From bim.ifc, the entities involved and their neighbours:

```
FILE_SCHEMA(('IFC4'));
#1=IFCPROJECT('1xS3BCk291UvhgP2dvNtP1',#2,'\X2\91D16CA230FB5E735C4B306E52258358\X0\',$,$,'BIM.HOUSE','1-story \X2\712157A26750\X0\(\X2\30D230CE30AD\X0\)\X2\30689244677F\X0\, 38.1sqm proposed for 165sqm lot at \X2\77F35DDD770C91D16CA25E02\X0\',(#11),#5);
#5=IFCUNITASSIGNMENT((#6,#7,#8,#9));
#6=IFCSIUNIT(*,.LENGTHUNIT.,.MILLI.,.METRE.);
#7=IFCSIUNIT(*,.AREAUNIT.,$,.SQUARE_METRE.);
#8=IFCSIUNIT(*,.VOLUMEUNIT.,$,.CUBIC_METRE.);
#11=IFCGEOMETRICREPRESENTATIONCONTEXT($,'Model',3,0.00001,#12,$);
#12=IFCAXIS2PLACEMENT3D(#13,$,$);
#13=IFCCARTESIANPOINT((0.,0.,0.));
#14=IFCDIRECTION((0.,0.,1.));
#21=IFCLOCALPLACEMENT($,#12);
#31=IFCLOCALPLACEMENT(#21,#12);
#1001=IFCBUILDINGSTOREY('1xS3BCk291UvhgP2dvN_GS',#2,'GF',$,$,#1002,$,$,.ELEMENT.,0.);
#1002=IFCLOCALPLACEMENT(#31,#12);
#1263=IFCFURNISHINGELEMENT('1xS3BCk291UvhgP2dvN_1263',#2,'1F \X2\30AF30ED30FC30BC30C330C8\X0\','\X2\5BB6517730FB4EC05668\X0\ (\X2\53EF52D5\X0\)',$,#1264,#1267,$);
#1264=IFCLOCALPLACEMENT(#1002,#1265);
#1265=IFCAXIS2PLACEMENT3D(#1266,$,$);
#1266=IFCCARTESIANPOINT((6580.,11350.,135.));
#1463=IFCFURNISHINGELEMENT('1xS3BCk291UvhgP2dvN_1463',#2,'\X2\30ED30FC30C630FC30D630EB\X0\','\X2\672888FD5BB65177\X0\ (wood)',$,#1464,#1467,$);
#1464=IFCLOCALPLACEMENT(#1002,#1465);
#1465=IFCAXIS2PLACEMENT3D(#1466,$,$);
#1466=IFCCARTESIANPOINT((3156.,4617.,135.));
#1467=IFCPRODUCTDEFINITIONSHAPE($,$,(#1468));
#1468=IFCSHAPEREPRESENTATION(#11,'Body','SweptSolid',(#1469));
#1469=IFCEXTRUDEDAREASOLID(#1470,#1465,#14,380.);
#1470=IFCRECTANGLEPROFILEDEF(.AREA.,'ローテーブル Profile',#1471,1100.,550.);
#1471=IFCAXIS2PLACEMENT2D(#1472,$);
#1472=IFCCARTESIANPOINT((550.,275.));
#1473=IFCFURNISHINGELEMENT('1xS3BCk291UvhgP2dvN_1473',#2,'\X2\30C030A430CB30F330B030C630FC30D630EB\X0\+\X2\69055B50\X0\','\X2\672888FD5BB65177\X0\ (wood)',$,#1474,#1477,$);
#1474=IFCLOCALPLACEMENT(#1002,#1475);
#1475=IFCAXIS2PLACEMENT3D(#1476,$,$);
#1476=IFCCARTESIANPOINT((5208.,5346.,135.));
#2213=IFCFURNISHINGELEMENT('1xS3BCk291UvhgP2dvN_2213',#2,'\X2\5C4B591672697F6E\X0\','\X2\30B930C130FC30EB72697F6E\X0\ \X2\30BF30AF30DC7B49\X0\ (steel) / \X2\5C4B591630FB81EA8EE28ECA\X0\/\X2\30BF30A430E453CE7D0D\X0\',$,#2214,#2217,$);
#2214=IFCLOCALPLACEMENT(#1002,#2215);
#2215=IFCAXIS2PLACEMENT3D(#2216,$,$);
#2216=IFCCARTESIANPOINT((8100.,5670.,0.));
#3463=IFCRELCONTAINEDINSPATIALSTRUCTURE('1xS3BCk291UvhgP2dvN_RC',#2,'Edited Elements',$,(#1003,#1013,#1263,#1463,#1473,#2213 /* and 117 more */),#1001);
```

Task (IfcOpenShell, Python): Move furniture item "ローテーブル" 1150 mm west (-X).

```python
import ifcopenshell
import ifcopenshell.api.geometry
import ifcopenshell.util.placement

model = ifcopenshell.open("bim.ifc")

item = model.by_guid("1xS3BCk291UvhgP2dvN_1463")
matrix = ifcopenshell.util.placement.get_local_placement(item.ObjectPlacement)
matrix[0, 3] -= 1150.0
ifcopenshell.api.geometry.edit_object_placement(model, product=item, matrix=matrix, is_si=False)

print(ifcopenshell.util.placement.get_local_placement(item.ObjectPlacement).round(3) + 0.0)

model.write("bim_rev.ifc")
```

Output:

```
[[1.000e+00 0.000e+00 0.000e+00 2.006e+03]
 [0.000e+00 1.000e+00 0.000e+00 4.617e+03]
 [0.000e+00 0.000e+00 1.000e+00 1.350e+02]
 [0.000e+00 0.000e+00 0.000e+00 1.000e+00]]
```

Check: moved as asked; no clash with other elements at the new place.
